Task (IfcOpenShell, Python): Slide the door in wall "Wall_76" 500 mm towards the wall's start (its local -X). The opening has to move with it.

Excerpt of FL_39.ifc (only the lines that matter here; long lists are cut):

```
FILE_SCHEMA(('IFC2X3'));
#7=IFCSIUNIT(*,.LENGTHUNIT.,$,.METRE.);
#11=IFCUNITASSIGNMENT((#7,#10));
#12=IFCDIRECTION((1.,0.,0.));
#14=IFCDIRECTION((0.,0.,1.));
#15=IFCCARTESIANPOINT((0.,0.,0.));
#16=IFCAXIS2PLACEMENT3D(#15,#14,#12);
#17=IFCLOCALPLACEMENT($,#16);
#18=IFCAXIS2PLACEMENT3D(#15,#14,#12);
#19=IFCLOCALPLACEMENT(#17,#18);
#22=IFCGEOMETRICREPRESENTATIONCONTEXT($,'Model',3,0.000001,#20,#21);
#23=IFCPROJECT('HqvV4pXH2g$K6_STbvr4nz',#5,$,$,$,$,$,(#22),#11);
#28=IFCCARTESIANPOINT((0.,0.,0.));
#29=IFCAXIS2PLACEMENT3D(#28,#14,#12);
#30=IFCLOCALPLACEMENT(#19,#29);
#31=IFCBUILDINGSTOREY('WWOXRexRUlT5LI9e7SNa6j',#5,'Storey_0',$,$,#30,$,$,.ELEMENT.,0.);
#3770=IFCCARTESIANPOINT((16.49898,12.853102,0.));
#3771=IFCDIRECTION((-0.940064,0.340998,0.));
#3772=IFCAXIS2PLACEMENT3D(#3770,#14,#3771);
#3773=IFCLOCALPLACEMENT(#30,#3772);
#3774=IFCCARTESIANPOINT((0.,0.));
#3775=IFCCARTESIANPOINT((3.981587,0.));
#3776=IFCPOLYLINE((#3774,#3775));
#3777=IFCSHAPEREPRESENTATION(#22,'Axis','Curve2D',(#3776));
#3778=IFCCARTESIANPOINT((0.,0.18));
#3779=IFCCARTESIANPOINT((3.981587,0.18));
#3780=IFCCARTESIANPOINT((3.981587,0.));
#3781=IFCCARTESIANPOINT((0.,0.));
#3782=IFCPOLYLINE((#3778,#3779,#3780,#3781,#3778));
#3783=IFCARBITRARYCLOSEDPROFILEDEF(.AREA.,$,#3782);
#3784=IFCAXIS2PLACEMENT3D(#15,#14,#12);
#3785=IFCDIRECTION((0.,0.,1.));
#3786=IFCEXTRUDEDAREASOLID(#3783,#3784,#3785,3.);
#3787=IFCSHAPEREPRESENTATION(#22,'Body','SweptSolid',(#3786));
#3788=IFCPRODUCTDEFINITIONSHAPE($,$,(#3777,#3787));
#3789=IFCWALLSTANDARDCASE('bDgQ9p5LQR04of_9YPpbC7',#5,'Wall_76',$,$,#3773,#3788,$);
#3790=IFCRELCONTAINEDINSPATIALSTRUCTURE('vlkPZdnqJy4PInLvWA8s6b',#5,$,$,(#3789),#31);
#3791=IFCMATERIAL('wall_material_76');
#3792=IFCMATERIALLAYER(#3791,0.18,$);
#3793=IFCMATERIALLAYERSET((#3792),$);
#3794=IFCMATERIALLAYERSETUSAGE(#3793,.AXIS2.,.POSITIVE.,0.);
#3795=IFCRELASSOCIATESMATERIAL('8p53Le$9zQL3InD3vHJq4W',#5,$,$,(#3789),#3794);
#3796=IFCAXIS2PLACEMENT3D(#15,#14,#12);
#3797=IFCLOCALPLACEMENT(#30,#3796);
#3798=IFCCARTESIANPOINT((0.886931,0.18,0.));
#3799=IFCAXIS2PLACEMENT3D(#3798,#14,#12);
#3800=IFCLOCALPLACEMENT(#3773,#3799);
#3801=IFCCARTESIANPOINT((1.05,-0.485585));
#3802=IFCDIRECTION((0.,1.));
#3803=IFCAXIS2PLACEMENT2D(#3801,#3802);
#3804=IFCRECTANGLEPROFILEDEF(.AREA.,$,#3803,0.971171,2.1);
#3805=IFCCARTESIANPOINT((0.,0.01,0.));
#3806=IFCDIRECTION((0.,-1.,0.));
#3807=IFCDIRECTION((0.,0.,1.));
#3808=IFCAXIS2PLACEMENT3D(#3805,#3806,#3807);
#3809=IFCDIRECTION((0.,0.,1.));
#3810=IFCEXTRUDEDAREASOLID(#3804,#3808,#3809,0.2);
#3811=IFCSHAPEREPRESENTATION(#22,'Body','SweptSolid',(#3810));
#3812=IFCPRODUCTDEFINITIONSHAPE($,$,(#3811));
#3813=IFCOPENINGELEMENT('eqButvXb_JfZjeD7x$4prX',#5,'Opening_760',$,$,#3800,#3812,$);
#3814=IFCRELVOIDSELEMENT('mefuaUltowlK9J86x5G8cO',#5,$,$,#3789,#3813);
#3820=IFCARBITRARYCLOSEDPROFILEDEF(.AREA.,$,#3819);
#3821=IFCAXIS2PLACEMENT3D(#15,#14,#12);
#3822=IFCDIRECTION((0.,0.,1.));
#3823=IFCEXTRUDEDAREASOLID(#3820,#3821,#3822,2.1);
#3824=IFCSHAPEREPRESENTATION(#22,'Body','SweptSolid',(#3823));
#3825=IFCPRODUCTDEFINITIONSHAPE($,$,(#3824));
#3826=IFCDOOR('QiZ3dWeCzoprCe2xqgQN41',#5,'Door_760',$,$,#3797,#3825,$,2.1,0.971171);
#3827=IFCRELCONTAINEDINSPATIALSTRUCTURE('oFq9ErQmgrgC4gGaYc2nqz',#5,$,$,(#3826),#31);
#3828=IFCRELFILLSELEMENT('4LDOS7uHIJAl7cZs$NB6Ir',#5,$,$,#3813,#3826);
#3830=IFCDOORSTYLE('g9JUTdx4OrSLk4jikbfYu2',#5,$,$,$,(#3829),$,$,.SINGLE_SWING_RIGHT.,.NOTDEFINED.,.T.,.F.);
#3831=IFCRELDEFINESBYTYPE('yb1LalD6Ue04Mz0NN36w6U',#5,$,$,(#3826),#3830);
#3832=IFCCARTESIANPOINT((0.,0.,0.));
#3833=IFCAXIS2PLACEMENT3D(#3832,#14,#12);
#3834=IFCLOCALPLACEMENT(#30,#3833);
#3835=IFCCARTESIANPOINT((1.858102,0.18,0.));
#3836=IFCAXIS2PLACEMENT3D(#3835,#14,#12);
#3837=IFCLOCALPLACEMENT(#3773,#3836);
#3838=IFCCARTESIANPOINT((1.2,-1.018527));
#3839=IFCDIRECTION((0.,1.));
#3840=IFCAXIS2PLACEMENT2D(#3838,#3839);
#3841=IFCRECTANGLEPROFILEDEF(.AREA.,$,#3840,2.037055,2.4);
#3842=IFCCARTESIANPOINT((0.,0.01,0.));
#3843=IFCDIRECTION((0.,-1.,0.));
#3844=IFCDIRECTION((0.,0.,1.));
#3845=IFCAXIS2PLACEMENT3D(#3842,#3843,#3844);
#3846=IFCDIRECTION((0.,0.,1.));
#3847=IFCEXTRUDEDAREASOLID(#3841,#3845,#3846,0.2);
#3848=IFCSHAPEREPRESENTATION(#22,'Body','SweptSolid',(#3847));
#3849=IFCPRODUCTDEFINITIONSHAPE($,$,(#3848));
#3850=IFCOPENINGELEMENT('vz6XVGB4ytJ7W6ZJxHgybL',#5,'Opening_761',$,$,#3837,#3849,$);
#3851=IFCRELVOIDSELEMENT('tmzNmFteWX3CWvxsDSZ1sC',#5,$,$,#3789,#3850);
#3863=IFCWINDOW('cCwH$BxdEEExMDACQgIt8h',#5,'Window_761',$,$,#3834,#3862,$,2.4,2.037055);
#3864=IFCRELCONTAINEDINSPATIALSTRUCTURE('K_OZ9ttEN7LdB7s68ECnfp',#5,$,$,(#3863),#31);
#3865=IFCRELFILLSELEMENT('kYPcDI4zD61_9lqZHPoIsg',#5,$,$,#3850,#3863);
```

```python
import ifcopenshell
import ifcopenshell.api.geometry
import ifcopenshell.util.placement
import ifcopenshell.util.unit

model = ifcopenshell.open("FL_39.ifc")
unit_scale = ifcopenshell.util.unit.calculate_unit_scale(model)

door = model.by_id(3826)
opening = door.FillsVoids[0].RelatingOpeningElement
wall = opening.VoidsElements[0].RelatingBuildingElement

wall_matrix = ifcopenshell.util.placement.get_local_placement(wall.ObjectPlacement)
shift = wall_matrix[:3, 0] * -0.5 / unit_scale
before = ifcopenshell.util.placement.get_local_placement(door.ObjectPlacement)[:3, 3].copy()

# The door is not placed relative to its opening, so move both.
for product in (opening, door):
    matrix = ifcopenshell.util.placement.get_local_placement(product.ObjectPlacement)
    matrix[:3, 3] += shift
    ifcopenshell.api.geometry.edit_object_placement(model, product=product, matrix=matrix, is_si=False)

after = ifcopenshell.util.placement.get_local_placement(door.ObjectPlacement)[:3, 3]
print("door moved by", (after - before).round(3) + 0.0)

model.write("FL_39_updated.ifc")
```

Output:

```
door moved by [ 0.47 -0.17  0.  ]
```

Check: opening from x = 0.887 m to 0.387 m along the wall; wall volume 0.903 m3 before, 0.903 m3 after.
